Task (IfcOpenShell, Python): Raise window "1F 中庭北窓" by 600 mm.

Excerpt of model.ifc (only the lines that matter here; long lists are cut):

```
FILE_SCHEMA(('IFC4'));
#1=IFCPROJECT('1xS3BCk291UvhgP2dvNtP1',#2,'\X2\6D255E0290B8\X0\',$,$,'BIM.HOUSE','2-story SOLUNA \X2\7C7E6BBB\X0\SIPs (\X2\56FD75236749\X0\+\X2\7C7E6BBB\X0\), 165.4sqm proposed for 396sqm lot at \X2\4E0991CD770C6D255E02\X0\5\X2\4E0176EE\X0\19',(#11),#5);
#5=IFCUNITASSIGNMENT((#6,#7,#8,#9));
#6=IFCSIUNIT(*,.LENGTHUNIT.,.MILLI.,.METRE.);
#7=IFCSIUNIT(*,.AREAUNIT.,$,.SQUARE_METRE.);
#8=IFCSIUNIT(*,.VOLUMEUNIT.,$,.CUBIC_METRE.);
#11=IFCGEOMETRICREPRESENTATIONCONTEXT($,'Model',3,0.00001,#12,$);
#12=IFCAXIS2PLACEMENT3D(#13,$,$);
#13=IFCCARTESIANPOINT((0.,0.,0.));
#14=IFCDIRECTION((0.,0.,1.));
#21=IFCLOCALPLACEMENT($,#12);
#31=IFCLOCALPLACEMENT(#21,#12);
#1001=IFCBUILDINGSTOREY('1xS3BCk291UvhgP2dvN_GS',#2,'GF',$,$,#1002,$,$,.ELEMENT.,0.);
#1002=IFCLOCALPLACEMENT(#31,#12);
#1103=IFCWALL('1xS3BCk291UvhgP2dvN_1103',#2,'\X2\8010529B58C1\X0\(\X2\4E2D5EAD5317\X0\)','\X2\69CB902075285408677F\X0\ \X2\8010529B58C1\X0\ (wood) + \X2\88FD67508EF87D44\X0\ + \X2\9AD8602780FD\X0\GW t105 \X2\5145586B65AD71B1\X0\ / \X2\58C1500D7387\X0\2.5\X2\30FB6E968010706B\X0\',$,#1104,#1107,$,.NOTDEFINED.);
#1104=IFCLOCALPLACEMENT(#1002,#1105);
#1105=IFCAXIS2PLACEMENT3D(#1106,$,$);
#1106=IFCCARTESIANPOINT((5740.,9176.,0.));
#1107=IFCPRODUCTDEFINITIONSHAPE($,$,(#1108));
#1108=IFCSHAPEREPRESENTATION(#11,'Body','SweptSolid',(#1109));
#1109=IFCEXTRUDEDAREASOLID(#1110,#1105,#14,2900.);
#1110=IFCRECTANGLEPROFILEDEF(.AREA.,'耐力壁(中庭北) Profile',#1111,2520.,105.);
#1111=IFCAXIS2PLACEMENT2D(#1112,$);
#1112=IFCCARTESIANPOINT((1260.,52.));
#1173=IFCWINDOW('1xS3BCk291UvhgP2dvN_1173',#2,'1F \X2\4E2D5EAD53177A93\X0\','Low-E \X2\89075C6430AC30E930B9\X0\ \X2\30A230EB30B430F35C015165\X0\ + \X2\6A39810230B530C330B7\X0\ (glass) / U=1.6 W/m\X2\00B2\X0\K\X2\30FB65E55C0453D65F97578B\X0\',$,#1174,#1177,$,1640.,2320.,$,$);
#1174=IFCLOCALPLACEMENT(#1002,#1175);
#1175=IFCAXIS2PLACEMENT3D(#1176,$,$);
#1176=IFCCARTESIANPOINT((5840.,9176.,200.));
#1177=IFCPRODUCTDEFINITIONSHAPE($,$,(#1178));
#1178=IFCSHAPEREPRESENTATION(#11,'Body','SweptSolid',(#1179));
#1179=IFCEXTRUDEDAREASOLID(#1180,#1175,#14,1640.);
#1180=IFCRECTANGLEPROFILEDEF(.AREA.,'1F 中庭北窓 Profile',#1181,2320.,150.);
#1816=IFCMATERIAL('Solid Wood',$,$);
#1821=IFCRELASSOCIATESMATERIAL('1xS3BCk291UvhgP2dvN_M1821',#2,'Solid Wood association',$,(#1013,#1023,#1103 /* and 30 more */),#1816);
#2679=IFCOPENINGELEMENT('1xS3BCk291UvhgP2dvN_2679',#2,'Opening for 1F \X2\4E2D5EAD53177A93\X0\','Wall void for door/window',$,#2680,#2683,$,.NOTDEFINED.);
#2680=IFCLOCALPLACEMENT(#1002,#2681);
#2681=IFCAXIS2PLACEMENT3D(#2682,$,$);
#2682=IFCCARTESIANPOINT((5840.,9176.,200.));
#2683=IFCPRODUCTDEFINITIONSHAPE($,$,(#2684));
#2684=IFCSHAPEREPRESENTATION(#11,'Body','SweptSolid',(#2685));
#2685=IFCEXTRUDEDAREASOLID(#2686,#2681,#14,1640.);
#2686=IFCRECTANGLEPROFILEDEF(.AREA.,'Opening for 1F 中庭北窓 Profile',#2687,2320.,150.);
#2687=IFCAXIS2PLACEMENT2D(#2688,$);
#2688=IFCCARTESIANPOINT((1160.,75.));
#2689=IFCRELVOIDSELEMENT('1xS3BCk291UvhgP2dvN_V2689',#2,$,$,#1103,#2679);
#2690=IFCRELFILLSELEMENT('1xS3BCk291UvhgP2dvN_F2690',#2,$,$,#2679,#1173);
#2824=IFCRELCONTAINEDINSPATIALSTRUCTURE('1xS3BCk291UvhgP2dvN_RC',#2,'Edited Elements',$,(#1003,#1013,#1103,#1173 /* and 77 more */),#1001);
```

```python
import numpy as np
import ifcopenshell
import ifcopenshell.api.geometry
import ifcopenshell.util.placement
import ifcopenshell.util.unit

model = ifcopenshell.open("model.ifc")
unit_scale = ifcopenshell.util.unit.calculate_unit_scale(model)

window = model.by_guid("1xS3BCk291UvhgP2dvN_1173")
opening = window.FillsVoids[0].RelatingOpeningElement
dz = 0.6 / unit_scale

shift = np.array([0.0, 0.0, dz])
# The window is not placed relative to its opening, so move both.
for product in (opening, window):
    matrix = ifcopenshell.util.placement.get_local_placement(product.ObjectPlacement)
    matrix[:3, 3] += shift
    ifcopenshell.api.geometry.edit_object_placement(model, product=product, matrix=matrix, is_si=False)

print(f"moved by {dz * unit_scale:+.3f} m")

model.write("model_v2.ifc")
```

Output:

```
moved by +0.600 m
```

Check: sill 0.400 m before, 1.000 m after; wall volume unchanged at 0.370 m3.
